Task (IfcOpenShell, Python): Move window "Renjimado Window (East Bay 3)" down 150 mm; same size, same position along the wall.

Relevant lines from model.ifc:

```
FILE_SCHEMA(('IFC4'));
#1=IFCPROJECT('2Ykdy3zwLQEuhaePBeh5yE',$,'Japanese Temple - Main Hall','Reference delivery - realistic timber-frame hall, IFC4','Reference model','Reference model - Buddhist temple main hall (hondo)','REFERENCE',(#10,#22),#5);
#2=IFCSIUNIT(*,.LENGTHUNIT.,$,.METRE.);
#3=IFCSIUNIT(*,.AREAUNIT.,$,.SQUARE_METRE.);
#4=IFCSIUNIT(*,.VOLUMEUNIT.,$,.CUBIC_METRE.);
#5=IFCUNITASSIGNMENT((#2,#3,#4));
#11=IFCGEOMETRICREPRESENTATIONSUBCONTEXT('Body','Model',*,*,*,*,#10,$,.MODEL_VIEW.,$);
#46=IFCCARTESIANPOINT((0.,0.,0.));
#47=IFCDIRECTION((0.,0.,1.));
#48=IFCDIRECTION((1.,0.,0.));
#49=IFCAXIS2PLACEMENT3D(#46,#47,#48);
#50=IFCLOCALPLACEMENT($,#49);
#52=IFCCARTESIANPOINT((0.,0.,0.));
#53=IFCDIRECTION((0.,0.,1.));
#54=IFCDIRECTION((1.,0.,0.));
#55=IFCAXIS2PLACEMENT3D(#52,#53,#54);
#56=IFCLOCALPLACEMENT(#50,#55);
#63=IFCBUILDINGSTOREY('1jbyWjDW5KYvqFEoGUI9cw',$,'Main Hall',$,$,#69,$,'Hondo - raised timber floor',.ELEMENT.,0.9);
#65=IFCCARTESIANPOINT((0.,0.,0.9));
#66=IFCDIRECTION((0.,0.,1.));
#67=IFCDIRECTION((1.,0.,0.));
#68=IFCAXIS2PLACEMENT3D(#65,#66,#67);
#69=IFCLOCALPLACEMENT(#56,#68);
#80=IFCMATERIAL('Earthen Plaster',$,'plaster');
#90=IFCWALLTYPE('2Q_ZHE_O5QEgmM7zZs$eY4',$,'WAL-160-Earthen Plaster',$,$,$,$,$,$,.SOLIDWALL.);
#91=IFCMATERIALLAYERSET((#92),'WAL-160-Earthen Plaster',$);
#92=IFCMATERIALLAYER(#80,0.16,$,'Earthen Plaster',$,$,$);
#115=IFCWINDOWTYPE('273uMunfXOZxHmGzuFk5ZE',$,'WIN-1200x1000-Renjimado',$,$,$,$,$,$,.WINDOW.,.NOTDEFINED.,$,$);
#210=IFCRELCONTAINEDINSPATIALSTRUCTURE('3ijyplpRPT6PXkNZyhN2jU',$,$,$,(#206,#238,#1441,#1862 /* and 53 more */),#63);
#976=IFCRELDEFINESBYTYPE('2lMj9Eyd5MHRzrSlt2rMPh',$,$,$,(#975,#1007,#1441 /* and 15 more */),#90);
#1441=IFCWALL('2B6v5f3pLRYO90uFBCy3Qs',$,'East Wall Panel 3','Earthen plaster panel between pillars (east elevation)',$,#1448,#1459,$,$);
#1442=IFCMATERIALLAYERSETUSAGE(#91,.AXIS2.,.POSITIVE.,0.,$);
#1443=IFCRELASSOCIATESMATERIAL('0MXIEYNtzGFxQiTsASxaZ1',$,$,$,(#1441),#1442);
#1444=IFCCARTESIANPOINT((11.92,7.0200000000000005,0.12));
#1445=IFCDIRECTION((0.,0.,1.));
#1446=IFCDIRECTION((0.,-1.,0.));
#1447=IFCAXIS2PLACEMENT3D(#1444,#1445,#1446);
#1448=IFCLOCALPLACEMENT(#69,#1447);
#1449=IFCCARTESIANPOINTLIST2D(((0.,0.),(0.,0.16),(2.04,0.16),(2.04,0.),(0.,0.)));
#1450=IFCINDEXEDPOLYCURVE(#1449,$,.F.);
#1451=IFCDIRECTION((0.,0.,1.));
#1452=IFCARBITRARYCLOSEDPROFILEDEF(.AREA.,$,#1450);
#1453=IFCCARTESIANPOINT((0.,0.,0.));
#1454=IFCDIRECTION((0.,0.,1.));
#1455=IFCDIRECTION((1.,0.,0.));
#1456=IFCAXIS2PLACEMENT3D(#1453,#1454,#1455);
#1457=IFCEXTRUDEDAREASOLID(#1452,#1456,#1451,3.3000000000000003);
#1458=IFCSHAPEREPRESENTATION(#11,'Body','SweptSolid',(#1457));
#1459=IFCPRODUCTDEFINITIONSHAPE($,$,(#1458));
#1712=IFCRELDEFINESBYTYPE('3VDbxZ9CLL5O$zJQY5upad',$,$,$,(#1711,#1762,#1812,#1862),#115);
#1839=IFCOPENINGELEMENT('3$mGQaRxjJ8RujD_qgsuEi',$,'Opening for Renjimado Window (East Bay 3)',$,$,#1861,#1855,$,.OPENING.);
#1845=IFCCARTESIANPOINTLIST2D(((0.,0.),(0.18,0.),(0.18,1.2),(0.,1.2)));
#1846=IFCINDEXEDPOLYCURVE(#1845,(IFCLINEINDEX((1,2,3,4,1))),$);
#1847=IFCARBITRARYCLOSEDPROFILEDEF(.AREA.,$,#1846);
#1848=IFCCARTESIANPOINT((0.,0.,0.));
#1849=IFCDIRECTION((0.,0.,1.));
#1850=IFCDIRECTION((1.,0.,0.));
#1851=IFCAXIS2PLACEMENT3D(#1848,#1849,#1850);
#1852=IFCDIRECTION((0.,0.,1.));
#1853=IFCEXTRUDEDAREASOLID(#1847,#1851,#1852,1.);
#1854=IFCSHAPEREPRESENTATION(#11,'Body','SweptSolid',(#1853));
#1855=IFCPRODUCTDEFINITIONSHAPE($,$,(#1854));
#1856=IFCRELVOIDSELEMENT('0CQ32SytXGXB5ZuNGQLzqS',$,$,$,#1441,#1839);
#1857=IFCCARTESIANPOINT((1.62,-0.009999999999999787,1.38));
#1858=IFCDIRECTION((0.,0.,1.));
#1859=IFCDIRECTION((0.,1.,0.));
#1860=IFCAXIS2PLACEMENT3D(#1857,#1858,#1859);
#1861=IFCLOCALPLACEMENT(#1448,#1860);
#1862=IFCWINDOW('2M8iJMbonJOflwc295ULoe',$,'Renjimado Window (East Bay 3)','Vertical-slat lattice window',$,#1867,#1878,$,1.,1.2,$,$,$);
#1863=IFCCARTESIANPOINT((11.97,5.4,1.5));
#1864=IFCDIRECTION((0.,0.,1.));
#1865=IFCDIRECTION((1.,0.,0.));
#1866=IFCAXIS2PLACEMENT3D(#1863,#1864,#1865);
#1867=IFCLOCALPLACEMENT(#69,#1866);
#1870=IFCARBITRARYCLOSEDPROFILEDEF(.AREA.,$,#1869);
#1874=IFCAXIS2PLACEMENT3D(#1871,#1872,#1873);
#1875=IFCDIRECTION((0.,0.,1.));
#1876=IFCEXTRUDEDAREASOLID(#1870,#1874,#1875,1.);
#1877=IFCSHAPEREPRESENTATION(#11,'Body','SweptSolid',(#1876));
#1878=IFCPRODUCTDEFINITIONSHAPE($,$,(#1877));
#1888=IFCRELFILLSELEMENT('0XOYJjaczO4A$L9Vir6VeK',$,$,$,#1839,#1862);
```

```python
import numpy as np
import ifcopenshell
import ifcopenshell.api.geometry
import ifcopenshell.util.placement
import ifcopenshell.util.unit

model = ifcopenshell.open("model.ifc")
unit_scale = ifcopenshell.util.unit.calculate_unit_scale(model)

window = model.by_id(1862)
opening = window.FillsVoids[0].RelatingOpeningElement
dz = -0.15 / unit_scale

shift = np.array([0.0, 0.0, dz])
# The window is not placed relative to its opening, so move both.
for product in (opening, window):
    matrix = ifcopenshell.util.placement.get_local_placement(product.ObjectPlacement)
    matrix[:3, 3] += shift
    ifcopenshell.api.geometry.edit_object_placement(model, product=product, matrix=matrix, is_si=False)

print(f"moved by {dz * unit_scale:+.3f} m")

model.write("model-out.ifc")
```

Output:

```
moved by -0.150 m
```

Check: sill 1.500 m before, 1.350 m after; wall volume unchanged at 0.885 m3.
